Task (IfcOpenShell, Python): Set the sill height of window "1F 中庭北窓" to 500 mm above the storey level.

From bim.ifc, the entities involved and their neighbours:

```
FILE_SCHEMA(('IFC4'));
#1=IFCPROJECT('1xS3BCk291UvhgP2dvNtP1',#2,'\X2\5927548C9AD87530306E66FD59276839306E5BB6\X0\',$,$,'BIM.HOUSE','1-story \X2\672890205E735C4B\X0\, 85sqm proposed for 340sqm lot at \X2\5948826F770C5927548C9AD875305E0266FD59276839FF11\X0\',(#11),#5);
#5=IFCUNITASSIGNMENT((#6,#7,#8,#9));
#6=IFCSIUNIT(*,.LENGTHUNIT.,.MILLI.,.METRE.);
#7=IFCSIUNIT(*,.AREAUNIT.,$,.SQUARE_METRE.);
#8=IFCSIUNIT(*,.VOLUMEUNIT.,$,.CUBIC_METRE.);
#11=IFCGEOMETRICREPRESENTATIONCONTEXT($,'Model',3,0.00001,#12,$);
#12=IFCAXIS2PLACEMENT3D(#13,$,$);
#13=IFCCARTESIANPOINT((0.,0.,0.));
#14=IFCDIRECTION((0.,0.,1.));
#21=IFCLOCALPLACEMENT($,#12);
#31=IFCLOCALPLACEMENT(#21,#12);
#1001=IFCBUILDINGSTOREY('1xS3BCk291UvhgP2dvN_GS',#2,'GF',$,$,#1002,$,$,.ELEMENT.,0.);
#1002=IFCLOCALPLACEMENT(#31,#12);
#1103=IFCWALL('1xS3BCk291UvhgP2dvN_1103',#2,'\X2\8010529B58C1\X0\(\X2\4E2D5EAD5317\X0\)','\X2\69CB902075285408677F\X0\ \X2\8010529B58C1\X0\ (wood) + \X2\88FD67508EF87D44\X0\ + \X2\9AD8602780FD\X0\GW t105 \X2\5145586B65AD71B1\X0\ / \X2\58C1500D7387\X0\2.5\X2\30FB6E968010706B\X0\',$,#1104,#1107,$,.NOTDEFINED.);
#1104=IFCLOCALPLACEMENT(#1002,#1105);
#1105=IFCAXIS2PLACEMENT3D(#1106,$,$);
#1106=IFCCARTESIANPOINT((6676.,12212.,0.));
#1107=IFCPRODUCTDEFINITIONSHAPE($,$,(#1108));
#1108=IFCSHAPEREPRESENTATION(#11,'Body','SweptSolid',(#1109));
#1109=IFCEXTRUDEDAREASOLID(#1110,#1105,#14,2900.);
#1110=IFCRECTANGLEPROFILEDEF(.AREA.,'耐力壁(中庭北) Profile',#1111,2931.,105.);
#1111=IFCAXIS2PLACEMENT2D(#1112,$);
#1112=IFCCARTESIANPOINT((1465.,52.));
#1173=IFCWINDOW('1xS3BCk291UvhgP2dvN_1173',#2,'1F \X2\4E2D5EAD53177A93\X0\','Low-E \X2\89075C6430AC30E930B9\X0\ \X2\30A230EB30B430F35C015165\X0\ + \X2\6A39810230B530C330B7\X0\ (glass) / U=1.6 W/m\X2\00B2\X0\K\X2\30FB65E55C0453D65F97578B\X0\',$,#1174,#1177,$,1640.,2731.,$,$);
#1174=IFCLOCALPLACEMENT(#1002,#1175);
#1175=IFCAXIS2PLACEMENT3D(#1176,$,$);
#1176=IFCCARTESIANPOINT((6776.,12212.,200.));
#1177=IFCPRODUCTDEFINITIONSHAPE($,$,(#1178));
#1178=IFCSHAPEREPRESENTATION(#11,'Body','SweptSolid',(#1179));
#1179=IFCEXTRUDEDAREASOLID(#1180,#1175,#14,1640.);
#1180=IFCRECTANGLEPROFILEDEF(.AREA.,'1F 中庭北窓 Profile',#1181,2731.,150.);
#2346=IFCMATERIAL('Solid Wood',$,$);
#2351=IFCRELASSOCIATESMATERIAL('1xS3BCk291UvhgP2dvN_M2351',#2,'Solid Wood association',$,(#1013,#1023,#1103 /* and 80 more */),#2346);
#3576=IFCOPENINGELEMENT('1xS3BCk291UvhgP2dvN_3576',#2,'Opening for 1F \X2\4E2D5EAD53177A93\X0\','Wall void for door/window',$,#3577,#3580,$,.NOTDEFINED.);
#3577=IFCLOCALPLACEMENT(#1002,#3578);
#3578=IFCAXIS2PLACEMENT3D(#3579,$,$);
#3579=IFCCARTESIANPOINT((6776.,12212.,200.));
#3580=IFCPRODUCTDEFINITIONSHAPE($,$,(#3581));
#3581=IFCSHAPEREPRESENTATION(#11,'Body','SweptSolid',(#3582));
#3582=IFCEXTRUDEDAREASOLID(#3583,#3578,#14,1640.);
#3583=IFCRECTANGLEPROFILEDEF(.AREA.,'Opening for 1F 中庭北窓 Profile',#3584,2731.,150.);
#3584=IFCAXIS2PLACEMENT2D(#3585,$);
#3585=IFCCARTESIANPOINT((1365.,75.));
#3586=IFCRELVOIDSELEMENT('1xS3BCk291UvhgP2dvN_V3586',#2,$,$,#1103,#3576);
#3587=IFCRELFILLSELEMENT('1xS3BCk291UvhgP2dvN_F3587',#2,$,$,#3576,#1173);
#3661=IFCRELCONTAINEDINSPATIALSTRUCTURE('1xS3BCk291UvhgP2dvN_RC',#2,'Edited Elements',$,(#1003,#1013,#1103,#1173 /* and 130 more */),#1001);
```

```python
import numpy as np
import ifcopenshell
import ifcopenshell.api.geometry
import ifcopenshell.geom
import ifcopenshell.util.element
import ifcopenshell.util.placement
import ifcopenshell.util.shape
import ifcopenshell.util.unit

model = ifcopenshell.open("bim.ifc")
unit_scale = ifcopenshell.util.unit.calculate_unit_scale(model)

window = model.by_id(1173)
opening = window.FillsVoids[0].RelatingOpeningElement
storey = ifcopenshell.util.element.get_container(window, ifc_class="IfcBuildingStorey")
level = ifcopenshell.util.placement.get_local_placement(storey.ObjectPlacement)[2, 3]

# The opening's origin need not be at the sill, so measure its lowest point.
shape = ifcopenshell.geom.create_shape(ifcopenshell.geom.settings(), opening)
bottom = ifcopenshell.util.shape.get_shape_bottom_elevation(shape, shape.geometry) / unit_scale
dz = level + 0.5 / unit_scale - bottom

shift = np.array([0.0, 0.0, dz])
# The window is not placed relative to its opening, so move both.
for product in (opening, window):
    matrix = ifcopenshell.util.placement.get_local_placement(product.ObjectPlacement)
    matrix[:3, 3] += shift
    ifcopenshell.api.geometry.edit_object_placement(model, product=product, matrix=matrix, is_si=False)

print(f"moved by {dz * unit_scale:+.3f} m")

model.write("bim_v2.ifc")
```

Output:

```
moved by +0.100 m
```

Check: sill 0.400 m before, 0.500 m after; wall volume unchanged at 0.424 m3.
